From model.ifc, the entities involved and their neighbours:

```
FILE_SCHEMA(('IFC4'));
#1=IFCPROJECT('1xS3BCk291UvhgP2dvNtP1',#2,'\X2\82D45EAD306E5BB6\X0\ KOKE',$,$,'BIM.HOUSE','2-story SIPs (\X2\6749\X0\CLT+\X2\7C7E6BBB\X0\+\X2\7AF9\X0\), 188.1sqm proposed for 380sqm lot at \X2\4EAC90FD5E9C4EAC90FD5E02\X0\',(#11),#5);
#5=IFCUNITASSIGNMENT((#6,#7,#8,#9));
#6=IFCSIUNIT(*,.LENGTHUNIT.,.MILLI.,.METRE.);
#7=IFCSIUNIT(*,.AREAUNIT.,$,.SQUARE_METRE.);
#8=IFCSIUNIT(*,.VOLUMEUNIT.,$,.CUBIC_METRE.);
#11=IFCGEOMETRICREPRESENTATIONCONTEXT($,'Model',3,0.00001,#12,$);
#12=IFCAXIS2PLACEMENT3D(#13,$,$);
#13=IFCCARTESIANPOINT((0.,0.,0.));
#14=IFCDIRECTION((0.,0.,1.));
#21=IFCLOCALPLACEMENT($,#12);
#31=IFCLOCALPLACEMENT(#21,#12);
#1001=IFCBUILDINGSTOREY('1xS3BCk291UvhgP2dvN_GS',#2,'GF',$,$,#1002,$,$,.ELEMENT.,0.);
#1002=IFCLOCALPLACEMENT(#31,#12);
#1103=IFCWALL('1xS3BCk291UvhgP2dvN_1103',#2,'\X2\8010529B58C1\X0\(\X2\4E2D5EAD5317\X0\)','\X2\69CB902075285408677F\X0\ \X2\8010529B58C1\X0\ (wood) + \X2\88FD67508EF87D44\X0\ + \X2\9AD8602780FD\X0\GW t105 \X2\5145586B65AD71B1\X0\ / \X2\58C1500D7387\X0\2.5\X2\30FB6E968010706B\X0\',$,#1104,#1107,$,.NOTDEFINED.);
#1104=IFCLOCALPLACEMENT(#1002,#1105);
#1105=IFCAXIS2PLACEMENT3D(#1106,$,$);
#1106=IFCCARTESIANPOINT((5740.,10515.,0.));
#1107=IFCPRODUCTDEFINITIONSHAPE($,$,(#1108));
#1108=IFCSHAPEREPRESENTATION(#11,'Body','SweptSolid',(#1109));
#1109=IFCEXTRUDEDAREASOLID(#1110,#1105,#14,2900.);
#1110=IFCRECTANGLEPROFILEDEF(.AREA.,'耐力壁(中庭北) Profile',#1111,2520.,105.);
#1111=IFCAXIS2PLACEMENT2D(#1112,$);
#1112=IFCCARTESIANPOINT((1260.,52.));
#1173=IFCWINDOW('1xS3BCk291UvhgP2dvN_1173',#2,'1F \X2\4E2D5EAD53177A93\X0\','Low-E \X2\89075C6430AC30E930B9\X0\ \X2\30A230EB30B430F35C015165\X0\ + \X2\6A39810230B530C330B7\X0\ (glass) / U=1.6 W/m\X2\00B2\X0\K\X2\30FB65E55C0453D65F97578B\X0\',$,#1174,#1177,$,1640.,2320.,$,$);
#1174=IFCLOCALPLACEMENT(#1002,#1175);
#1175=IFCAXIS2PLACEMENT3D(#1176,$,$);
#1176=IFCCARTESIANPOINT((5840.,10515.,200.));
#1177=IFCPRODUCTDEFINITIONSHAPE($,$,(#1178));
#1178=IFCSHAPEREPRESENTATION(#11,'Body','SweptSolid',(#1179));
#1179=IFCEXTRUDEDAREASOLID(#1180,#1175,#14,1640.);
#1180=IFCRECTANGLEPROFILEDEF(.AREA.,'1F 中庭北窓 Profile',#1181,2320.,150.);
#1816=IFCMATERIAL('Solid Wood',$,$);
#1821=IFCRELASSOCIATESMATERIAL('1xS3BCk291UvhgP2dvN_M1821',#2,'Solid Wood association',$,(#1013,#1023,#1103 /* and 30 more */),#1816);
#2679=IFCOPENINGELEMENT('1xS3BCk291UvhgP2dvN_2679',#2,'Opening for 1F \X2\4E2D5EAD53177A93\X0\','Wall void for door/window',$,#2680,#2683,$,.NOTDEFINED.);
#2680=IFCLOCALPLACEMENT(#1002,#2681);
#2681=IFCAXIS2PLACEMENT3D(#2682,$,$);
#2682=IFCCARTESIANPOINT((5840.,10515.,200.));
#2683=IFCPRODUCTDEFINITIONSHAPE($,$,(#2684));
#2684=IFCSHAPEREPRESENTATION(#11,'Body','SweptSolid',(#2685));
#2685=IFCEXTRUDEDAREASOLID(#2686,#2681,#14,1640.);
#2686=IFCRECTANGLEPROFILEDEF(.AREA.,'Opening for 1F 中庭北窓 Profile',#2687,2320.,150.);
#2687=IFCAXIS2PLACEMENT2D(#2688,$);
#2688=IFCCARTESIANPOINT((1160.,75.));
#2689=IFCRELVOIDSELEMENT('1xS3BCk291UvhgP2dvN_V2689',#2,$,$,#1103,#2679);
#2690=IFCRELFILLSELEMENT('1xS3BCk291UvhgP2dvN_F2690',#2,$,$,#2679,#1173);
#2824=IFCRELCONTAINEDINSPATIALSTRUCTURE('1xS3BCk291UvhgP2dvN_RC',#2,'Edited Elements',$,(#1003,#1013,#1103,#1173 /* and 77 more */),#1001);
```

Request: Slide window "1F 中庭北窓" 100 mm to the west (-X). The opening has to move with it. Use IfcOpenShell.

```python
import ifcopenshell
import ifcopenshell.api.geometry
import ifcopenshell.util.placement
import ifcopenshell.util.unit

model = ifcopenshell.open("model.ifc")
unit_scale = ifcopenshell.util.unit.calculate_unit_scale(model)

window = model.by_guid("1xS3BCk291UvhgP2dvN_1173")
opening = window.FillsVoids[0].RelatingOpeningElement
wall = opening.VoidsElements[0].RelatingBuildingElement

wall_matrix = ifcopenshell.util.placement.get_local_placement(wall.ObjectPlacement)
shift = wall_matrix[:3, 0] * -0.1 / unit_scale
before = ifcopenshell.util.placement.get_local_placement(window.ObjectPlacement)[:3, 3].copy()

# The window is not placed relative to its opening, so move both.
for product in (opening, window):
    matrix = ifcopenshell.util.placement.get_local_placement(product.ObjectPlacement)
    matrix[:3, 3] += shift
    ifcopenshell.api.geometry.edit_object_placement(model, product=product, matrix=matrix, is_si=False)

after = ifcopenshell.util.placement.get_local_placement(window.ObjectPlacement)[:3, 3]
print("window moved by", (after - before).round(3) + 0.0)

model.write("model_rev.ifc")
```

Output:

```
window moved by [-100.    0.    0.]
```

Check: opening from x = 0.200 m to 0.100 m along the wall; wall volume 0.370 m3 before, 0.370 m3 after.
